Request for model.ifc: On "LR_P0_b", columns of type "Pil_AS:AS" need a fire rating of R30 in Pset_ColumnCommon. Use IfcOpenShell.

First a look at what the model holds.

```python
import ifcopenshell
import ifcopenshell.util.element

model = ifcopenshell.open("model.ifc")
print(model.schema)
storey = next(s for s in model.by_type("IfcBuildingStorey") if s.Name == "LR_P0_b")
columns = [e for e in ifcopenshell.util.element.get_decomposition(storey) if e.is_a("IfcColumn")]
seen = {}
for e in columns:
    element_type = ifcopenshell.util.element.get_type(e)
    key = (element_type.Name if element_type != e and element_type else None, ifcopenshell.util.element.get_pset(e, "Pset_ColumnCommon", "FireRating"))
    seen[key] = seen.get(key, 0) + 1
for (name, value), count in sorted(seen.items(), key=str):
    print(count, "x", name, "|", value)
```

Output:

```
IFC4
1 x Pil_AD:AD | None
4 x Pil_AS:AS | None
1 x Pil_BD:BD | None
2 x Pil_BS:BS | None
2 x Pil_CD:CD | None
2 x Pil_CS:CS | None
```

```python
import ifcopenshell
import ifcopenshell.api.pset
import ifcopenshell.util.element

model = ifcopenshell.open("model.ifc")

storey = next(s for s in model.by_type("IfcBuildingStorey") if s.Name == "LR_P0_b")
columns = [e for e in ifcopenshell.util.element.get_decomposition(storey) if e.is_a("IfcColumn")]

count = 0
for e in columns:
    element_type = ifcopenshell.util.element.get_type(e)
    if element_type in (None, e) or element_type.Name != "Pil_AS:AS":
        continue
    # add_pset returns the element's existing set when there is one.
    pset = ifcopenshell.api.pset.add_pset(model, product=e, name="Pset_ColumnCommon")
    ifcopenshell.api.pset.edit_pset(model, pset=pset, properties={"FireRating": "R30"})
    count += 1

print(count, "columns updated")

model.write("model_v2.ifc")
```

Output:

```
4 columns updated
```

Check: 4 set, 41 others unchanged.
